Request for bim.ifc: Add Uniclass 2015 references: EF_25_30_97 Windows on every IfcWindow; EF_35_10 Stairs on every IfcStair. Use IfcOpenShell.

First a look at what the model holds.

```python
import ifcopenshell

model = ifcopenshell.open("bim.ifc")
print(model.schema)
print("classifications:", [c.Name for c in model.by_type("IfcClassification")])
for ifc_class in ("IfcDoor", "IfcRoof", "IfcStair", "IfcWall", "IfcWindow"):
    print(ifc_class, len(model.by_type(ifc_class)))
```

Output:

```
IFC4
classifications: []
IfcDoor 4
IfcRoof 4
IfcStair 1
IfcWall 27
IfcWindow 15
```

```python
import ifcopenshell
import ifcopenshell.api.classification

model = ifcopenshell.open("bim.ifc")

system = ifcopenshell.api.classification.add_classification(model, classification="Uniclass 2015")

codes = {
    "IfcWindow": ("EF_25_30_97", "Windows"),
    "IfcStair": ("EF_35_10", "Stairs"),
}
for ifc_class, (code, name) in codes.items():
    products = model.by_type(ifc_class)
    ifcopenshell.api.classification.add_reference(
        model, products=products, classification=system, identification=code, name=name
    )
    print(code, len(products))

model.write("bim_edited.ifc")
```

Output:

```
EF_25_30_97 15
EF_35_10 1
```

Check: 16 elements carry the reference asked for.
